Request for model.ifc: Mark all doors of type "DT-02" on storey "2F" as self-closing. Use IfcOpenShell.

First a look at what the model holds.

```python
import ifcopenshell
import ifcopenshell.util.element

model = ifcopenshell.open("model.ifc")
print(model.schema)
storey = next(s for s in model.by_type("IfcBuildingStorey") if s.Name == "2F")
doors = [e for e in ifcopenshell.util.element.get_decomposition(storey) if e.is_a("IfcDoor")]
seen = {}
for e in doors:
    element_type = ifcopenshell.util.element.get_type(e)
    key = (element_type.Name if element_type != e and element_type else None, ifcopenshell.util.element.get_pset(e, "Pset_DoorCommon", "SelfClosing"))
    seen[key] = seen.get(key, 0) + 1
for (name, value), count in sorted(seen.items(), key=str):
    print(count, "x", name, "|", value)
```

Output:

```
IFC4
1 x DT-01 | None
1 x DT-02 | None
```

```python
import ifcopenshell
import ifcopenshell.api.pset
import ifcopenshell.util.element

model = ifcopenshell.open("model.ifc")

storey = next(s for s in model.by_type("IfcBuildingStorey") if s.Name == "2F")
doors = [e for e in ifcopenshell.util.element.get_decomposition(storey) if e.is_a("IfcDoor")]

count = 0
for e in doors:
    element_type = ifcopenshell.util.element.get_type(e)
    if element_type in (None, e) or element_type.Name != "DT-02":
        continue
    # add_pset returns the element's existing set when there is one.
    pset = ifcopenshell.api.pset.add_pset(model, product=e, name="Pset_DoorCommon")
    ifcopenshell.api.pset.edit_pset(model, pset=pset, properties={"SelfClosing": True})
    count += 1

print(count, "doors updated")

model.write("model_updated.ifc")
```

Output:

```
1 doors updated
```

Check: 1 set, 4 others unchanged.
